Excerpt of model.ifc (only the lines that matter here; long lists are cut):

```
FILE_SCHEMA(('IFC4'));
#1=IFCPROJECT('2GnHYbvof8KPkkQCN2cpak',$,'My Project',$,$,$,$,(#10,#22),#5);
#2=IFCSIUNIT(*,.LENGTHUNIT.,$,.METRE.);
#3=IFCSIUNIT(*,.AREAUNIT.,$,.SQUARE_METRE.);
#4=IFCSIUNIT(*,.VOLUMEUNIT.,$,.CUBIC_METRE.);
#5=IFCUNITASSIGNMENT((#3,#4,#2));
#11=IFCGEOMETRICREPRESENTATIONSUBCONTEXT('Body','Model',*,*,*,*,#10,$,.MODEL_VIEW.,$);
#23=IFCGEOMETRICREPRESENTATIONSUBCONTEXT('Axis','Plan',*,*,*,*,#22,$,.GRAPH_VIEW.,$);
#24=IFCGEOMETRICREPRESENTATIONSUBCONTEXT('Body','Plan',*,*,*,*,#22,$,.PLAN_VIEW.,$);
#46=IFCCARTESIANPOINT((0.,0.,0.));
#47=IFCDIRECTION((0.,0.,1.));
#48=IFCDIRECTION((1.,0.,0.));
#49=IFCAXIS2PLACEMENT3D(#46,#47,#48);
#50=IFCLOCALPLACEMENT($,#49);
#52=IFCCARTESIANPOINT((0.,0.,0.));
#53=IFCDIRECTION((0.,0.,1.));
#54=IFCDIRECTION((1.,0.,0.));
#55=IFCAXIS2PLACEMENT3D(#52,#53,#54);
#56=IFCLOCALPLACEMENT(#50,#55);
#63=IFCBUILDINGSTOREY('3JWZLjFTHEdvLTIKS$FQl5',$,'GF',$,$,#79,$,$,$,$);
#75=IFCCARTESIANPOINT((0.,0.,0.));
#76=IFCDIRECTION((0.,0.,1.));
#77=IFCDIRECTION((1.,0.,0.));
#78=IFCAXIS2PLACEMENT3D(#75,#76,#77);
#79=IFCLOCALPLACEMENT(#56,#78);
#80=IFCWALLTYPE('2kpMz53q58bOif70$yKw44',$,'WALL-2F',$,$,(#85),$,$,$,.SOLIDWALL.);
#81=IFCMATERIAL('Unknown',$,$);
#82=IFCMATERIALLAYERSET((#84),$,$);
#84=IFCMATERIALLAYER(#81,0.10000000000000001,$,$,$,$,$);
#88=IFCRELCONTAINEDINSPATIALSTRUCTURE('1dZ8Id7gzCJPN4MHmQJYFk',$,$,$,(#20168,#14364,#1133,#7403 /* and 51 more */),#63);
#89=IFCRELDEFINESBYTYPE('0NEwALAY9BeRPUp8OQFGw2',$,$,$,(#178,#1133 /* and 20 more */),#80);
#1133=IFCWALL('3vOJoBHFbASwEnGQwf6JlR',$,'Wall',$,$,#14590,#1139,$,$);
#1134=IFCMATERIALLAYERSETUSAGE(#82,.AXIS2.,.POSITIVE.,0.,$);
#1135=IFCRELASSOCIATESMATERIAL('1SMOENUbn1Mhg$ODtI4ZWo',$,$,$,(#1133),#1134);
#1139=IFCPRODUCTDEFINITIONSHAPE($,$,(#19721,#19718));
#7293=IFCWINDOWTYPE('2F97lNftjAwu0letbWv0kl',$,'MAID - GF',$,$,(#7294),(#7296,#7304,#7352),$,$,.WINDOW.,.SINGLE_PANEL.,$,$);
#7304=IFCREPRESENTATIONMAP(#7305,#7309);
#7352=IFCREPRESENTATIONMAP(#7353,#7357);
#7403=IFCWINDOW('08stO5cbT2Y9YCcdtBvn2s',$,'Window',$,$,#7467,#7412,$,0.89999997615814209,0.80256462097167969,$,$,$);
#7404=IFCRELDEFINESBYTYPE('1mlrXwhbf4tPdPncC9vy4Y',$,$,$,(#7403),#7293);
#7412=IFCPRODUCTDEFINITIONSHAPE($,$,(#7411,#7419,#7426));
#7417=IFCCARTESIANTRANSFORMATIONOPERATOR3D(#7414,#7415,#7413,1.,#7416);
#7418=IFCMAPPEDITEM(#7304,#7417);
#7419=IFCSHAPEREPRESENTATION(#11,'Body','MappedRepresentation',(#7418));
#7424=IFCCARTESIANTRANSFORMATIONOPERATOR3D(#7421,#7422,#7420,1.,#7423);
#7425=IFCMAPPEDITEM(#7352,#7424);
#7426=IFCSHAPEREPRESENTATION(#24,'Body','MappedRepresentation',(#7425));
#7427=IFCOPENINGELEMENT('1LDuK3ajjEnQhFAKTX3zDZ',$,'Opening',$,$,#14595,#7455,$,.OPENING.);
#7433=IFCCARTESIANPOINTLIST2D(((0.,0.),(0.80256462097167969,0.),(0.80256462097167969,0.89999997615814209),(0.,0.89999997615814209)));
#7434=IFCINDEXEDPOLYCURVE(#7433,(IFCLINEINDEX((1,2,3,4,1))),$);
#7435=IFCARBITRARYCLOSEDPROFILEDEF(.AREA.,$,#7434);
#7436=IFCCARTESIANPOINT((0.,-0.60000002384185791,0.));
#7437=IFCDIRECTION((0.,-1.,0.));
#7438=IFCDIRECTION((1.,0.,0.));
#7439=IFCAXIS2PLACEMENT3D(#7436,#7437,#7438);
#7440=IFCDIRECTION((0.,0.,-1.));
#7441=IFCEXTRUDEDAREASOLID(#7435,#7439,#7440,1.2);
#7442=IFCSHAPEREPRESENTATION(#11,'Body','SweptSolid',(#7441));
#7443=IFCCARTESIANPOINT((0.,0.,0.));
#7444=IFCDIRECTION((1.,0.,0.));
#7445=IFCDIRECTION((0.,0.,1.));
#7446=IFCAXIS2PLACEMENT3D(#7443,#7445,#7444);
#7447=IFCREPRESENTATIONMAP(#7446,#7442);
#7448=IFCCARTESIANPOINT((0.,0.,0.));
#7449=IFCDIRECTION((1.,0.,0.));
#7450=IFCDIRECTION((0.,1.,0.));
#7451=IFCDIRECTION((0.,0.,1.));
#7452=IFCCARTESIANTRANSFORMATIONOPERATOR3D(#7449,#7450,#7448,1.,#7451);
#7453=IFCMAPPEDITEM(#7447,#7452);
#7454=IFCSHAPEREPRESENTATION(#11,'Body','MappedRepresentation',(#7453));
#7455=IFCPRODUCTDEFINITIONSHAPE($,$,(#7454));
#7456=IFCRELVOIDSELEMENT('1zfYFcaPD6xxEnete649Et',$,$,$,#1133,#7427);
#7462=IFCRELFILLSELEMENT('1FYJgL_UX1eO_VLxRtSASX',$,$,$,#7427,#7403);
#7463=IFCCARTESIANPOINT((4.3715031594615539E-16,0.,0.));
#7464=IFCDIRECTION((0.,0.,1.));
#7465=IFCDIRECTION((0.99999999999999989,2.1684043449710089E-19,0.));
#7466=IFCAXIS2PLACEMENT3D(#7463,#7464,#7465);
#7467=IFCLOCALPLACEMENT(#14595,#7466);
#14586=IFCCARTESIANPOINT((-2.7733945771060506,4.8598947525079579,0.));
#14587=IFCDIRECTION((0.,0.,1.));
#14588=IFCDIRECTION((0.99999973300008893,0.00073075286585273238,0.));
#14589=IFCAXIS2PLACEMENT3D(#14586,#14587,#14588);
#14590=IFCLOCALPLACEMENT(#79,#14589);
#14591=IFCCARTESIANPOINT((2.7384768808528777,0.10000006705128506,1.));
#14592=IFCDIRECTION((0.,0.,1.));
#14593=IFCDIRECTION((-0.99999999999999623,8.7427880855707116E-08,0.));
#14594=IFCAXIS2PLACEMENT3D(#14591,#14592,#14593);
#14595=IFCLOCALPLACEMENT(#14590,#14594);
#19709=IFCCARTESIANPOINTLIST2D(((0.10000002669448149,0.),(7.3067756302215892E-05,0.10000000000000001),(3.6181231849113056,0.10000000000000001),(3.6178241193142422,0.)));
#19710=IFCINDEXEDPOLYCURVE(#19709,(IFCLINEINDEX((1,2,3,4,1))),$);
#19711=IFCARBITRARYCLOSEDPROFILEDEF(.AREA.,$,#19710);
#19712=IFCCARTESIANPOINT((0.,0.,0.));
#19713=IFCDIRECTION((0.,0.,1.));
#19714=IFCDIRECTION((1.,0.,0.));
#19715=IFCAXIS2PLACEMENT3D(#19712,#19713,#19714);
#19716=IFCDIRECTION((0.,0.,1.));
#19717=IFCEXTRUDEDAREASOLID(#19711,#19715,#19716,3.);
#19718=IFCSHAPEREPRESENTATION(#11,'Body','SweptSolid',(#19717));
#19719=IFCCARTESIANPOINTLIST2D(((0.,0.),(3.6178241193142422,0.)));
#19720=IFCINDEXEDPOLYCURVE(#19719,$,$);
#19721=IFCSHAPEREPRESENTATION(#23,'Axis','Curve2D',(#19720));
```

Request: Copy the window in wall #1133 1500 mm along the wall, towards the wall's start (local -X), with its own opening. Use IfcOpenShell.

```python
import ifcopenshell
import ifcopenshell.api.feature
import ifcopenshell.api.geometry
import ifcopenshell.api.root
import ifcopenshell.geom
import ifcopenshell.util.element
import ifcopenshell.util.placement
import ifcopenshell.util.shape

model = ifcopenshell.open("model.ifc")
settings = ifcopenshell.geom.settings()


def volume(element):
    """Net volume in cubic metres, openings subtracted."""
    shape = ifcopenshell.geom.create_shape(settings, element)
    return ifcopenshell.util.shape.get_volume(shape.geometry)


window = model.by_guid("08stO5cbT2Y9YCcdtBvn2s")
opening = window.FillsVoids[0].RelatingOpeningElement
wall = opening.VoidsElements[0].RelatingBuildingElement
before = volume(wall)
shift = ifcopenshell.util.placement.get_local_placement(wall.ObjectPlacement)[:3, 0] * -1.5

# copy_class copies the void relationship, type, container and properties, but no geometry.
new_opening = ifcopenshell.api.root.copy_class(model, product=opening)
new_opening.Representation = ifcopenshell.util.element.copy_deep(
    model, opening.Representation, exclude=["IfcGeometricRepresentationContext", "IfcRepresentationMap"]
)
new_window = ifcopenshell.api.root.copy_class(model, product=window)
new_window.Representation = ifcopenshell.util.element.copy_deep(
    model, window.Representation, exclude=["IfcGeometricRepresentationContext", "IfcRepresentationMap"]
)
ifcopenshell.api.feature.add_filling(model, opening=new_opening, element=new_window)

for old, new in ((opening, new_opening), (window, new_window)):
    matrix = ifcopenshell.util.placement.get_local_placement(old.ObjectPlacement)
    matrix[:3, 3] += shift
    ifcopenshell.api.geometry.edit_object_placement(model, product=new, matrix=matrix, is_si=False)

after = volume(wall)

print(f"wall volume {before:.3f} -> {after:.3f} m3")

model.write("model_rev.ifc")
```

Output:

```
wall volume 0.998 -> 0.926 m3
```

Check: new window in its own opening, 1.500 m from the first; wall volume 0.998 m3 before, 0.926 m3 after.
